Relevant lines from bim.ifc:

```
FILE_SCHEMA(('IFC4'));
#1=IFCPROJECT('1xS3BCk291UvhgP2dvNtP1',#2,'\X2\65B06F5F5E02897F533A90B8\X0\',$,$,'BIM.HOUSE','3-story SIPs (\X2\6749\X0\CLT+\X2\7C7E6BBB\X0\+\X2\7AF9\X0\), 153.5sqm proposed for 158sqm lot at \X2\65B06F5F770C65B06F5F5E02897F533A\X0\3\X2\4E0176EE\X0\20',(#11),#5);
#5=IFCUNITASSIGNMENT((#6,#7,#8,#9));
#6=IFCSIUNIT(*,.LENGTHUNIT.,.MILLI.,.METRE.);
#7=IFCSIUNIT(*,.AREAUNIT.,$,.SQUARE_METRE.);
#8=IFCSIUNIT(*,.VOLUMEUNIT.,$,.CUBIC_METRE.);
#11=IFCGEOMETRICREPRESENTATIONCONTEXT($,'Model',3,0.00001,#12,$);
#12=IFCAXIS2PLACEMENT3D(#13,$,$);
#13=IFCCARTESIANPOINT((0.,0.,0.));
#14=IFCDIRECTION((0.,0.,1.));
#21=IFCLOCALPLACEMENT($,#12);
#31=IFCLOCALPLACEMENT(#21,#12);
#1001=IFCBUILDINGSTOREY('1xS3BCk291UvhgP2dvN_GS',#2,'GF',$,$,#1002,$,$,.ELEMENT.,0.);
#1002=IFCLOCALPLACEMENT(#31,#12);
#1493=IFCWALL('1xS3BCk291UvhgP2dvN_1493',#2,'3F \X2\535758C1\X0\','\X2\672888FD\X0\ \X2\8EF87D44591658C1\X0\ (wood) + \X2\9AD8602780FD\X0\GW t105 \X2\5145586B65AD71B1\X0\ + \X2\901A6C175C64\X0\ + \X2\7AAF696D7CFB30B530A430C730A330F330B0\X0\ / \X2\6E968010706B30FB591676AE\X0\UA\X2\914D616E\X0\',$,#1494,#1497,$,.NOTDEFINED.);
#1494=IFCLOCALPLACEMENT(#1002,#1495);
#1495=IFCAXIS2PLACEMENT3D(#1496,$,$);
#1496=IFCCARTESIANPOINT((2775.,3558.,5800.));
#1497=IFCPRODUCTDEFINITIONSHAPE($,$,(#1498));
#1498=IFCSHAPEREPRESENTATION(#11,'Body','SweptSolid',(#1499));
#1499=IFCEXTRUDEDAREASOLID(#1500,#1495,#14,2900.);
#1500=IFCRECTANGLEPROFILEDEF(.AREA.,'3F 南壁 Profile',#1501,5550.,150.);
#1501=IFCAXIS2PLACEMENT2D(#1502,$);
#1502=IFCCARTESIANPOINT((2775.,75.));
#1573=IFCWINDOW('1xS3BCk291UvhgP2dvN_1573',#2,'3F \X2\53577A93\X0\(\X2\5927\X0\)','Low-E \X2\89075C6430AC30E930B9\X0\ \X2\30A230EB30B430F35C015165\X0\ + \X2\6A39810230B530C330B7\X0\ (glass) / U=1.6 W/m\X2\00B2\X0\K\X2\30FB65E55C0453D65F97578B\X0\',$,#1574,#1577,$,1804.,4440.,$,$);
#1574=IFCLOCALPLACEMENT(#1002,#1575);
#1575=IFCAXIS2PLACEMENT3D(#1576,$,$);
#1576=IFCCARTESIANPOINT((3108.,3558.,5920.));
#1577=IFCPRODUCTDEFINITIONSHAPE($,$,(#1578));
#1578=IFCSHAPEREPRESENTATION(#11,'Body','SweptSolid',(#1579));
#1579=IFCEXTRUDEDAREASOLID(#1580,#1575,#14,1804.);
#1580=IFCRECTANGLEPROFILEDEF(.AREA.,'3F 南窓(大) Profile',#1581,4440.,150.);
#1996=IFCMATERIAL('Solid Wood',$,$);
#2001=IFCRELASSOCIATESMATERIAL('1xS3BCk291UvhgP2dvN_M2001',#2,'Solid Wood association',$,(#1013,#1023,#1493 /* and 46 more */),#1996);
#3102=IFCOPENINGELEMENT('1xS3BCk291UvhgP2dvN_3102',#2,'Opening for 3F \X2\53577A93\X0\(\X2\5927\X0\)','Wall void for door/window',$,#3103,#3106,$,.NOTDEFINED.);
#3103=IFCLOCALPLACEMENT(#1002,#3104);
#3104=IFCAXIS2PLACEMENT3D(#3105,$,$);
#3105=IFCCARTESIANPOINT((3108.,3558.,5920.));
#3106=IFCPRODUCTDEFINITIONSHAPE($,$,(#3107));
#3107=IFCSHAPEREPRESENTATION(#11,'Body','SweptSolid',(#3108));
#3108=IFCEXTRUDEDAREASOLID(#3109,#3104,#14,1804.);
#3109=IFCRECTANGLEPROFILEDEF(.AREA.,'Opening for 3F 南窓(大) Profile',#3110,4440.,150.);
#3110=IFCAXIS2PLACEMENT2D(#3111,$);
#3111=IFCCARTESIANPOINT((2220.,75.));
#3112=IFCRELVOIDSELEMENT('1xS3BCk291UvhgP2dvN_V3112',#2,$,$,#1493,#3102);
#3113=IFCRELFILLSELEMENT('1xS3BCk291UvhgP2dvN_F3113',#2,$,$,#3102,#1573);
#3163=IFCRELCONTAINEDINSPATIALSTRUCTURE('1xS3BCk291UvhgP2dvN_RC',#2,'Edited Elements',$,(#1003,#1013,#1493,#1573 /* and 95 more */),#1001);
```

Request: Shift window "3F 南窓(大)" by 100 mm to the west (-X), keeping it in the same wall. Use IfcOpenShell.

```python
import ifcopenshell
import ifcopenshell.api.geometry
import ifcopenshell.util.placement

model = ifcopenshell.open("bim.ifc")

window = model.by_guid("1xS3BCk291UvhgP2dvN_1573")
opening = window.FillsVoids[0].RelatingOpeningElement
wall = opening.VoidsElements[0].RelatingBuildingElement

wall_matrix = ifcopenshell.util.placement.get_local_placement(wall.ObjectPlacement)
shift = wall_matrix[:3, 0] * -100.0
before = ifcopenshell.util.placement.get_local_placement(window.ObjectPlacement)[:3, 3].copy()

# The window is not placed relative to its opening, so move both.
for product in (opening, window):
    matrix = ifcopenshell.util.placement.get_local_placement(product.ObjectPlacement)
    matrix[:3, 3] += shift
    ifcopenshell.api.geometry.edit_object_placement(model, product=product, matrix=matrix, is_si=False)

after = ifcopenshell.util.placement.get_local_placement(window.ObjectPlacement)[:3, 3]
print("window moved by", (after - before).round(3) + 0.0)

model.write("bim_v2.ifc")
```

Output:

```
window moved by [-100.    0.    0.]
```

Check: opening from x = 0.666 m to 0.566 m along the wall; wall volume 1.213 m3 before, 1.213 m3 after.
